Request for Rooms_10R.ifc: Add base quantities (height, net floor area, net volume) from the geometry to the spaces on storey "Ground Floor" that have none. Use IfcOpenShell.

First a look at what the model holds.

```python
import ifcopenshell
import ifcopenshell.util.element
import ifcopenshell.util.unit

model = ifcopenshell.open("Rooms_10R.ifc")
print(model.schema)
for unit_type in ("LENGTHUNIT", "AREAUNIT", "VOLUMEUNIT"):
    print(unit_type, ifcopenshell.util.unit.calculate_unit_scale(model, unit_type))
storey = next(s for s in model.by_type("IfcBuildingStorey") if s.Name == "Ground Floor")
spaces = [e for e in ifcopenshell.util.element.get_decomposition(storey) if e.is_a("IfcSpace")]
for e in sorted(spaces, key=lambda e: e.id()):
    print(e.id(), e.is_a(), e.Name, list(ifcopenshell.util.element.get_psets(e, qtos_only=True)), sep=" | ")
```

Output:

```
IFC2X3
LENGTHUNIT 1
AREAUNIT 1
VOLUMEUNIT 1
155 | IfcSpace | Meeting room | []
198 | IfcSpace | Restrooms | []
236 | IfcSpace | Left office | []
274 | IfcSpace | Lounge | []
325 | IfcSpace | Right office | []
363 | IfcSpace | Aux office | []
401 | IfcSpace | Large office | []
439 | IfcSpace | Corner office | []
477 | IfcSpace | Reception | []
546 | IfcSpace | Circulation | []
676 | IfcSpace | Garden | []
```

```python
import ifcopenshell
import ifcopenshell.api.pset
import ifcopenshell.geom
import ifcopenshell.util.element
import ifcopenshell.util.shape
import ifcopenshell.util.unit

model = ifcopenshell.open("Rooms_10R.ifc")
unit_scale = ifcopenshell.util.unit.calculate_unit_scale(model)
area_scale = ifcopenshell.util.unit.calculate_unit_scale(model, "AREAUNIT")
volume_scale = ifcopenshell.util.unit.calculate_unit_scale(model, "VOLUMEUNIT")
settings = ifcopenshell.geom.settings()

storey = next(s for s in model.by_type("IfcBuildingStorey") if s.Name == "Ground Floor")
spaces = [e for e in ifcopenshell.util.element.get_decomposition(storey) if e.is_a("IfcSpace")]

for e in sorted(spaces, key=lambda e: e.id()):
    if ifcopenshell.util.element.get_psets(e, qtos_only=True, should_inherit=False):
        continue
    # Geometry comes back in metres, in the element's own axes.
    shape = ifcopenshell.geom.create_shape(settings, e)
    values = {
        "Height": ifcopenshell.util.shape.get_z(shape.geometry) / unit_scale,
        "NetFloorArea": ifcopenshell.util.shape.get_footprint_area(shape.geometry) / area_scale,
        "NetVolume": ifcopenshell.util.shape.get_volume(shape.geometry) / volume_scale,
    }
    qto = ifcopenshell.api.pset.add_qto(model, product=e, name="BaseQuantities")
    ifcopenshell.api.pset.edit_qto(model, qto=qto, properties=values)
    print(e.id(), {k: round(v, 3) for k, v in values.items()})

model.write("Rooms_10R_updated.ifc")
```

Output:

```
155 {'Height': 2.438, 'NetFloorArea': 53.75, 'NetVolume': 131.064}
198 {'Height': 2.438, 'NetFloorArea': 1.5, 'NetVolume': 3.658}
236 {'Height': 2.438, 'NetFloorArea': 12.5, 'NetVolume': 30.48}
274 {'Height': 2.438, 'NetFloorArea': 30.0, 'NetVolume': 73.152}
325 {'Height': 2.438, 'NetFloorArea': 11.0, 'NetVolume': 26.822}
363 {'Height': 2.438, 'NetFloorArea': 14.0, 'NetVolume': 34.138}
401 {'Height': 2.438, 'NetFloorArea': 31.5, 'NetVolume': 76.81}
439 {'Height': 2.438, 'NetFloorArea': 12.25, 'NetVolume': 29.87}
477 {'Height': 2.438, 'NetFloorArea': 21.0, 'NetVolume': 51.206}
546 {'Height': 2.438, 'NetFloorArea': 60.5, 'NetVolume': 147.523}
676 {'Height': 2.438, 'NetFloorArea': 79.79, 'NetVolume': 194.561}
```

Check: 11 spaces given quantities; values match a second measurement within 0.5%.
